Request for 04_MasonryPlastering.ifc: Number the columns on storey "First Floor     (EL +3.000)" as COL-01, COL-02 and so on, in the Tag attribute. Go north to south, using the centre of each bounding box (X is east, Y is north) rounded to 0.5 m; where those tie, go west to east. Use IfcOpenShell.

First a look at what the model holds.

```python
import ifcopenshell
import ifcopenshell.util.element
import ifcopenshell.util.placement

model = ifcopenshell.open("04_MasonryPlastering.ifc")
print(model.schema)
storey = next(s for s in model.by_type("IfcBuildingStorey") if s.Name == "First Floor     (EL +3.000)")
columns = [e for e in ifcopenshell.util.element.get_decomposition(storey) if e.is_a("IfcColumn")]
for e in sorted(columns, key=lambda e: e.id()):
    origin = ifcopenshell.util.placement.get_local_placement(e.ObjectPlacement)[:3, 3]
    print(e.id(), e.Tag, e.Name, origin.round(2) + 0.0, sep=" | ")
```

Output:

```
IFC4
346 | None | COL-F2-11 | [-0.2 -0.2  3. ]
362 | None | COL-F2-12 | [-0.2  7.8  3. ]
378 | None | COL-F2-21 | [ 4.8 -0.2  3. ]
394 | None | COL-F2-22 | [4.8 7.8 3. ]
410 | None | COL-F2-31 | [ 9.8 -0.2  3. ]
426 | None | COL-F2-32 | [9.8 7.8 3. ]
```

```python
import ifcopenshell
import ifcopenshell.geom
import ifcopenshell.util.element
import ifcopenshell.util.shape

model = ifcopenshell.open("04_MasonryPlastering.ifc")
settings = ifcopenshell.geom.settings()
settings.set("use-world-coords", True)


def centre(element):
    shape = ifcopenshell.geom.create_shape(settings, element)
    return ifcopenshell.util.shape.get_bbox_centroid(shape.geometry)


storey = next(s for s in model.by_type("IfcBuildingStorey") if s.Name == "First Floor     (EL +3.000)")
columns = [e for e in ifcopenshell.util.element.get_decomposition(storey) if e.is_a("IfcColumn")]

# Insertion points can sit at a corner or the storey origin, so sort by the geometry (in metres).
centres = {e: centre(e) for e in columns}
columns.sort(key=lambda e: (-round(centres[e][1] / 0.5), centres[e][0]))

for i, e in enumerate(columns, start=1):
    number = f"COL-{i:02d}"
    e.Tag = number
    print(e.id(), number)

model.write("04_MasonryPlastering_rev.ifc")
```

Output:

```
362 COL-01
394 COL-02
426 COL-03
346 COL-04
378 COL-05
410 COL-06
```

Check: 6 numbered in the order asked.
